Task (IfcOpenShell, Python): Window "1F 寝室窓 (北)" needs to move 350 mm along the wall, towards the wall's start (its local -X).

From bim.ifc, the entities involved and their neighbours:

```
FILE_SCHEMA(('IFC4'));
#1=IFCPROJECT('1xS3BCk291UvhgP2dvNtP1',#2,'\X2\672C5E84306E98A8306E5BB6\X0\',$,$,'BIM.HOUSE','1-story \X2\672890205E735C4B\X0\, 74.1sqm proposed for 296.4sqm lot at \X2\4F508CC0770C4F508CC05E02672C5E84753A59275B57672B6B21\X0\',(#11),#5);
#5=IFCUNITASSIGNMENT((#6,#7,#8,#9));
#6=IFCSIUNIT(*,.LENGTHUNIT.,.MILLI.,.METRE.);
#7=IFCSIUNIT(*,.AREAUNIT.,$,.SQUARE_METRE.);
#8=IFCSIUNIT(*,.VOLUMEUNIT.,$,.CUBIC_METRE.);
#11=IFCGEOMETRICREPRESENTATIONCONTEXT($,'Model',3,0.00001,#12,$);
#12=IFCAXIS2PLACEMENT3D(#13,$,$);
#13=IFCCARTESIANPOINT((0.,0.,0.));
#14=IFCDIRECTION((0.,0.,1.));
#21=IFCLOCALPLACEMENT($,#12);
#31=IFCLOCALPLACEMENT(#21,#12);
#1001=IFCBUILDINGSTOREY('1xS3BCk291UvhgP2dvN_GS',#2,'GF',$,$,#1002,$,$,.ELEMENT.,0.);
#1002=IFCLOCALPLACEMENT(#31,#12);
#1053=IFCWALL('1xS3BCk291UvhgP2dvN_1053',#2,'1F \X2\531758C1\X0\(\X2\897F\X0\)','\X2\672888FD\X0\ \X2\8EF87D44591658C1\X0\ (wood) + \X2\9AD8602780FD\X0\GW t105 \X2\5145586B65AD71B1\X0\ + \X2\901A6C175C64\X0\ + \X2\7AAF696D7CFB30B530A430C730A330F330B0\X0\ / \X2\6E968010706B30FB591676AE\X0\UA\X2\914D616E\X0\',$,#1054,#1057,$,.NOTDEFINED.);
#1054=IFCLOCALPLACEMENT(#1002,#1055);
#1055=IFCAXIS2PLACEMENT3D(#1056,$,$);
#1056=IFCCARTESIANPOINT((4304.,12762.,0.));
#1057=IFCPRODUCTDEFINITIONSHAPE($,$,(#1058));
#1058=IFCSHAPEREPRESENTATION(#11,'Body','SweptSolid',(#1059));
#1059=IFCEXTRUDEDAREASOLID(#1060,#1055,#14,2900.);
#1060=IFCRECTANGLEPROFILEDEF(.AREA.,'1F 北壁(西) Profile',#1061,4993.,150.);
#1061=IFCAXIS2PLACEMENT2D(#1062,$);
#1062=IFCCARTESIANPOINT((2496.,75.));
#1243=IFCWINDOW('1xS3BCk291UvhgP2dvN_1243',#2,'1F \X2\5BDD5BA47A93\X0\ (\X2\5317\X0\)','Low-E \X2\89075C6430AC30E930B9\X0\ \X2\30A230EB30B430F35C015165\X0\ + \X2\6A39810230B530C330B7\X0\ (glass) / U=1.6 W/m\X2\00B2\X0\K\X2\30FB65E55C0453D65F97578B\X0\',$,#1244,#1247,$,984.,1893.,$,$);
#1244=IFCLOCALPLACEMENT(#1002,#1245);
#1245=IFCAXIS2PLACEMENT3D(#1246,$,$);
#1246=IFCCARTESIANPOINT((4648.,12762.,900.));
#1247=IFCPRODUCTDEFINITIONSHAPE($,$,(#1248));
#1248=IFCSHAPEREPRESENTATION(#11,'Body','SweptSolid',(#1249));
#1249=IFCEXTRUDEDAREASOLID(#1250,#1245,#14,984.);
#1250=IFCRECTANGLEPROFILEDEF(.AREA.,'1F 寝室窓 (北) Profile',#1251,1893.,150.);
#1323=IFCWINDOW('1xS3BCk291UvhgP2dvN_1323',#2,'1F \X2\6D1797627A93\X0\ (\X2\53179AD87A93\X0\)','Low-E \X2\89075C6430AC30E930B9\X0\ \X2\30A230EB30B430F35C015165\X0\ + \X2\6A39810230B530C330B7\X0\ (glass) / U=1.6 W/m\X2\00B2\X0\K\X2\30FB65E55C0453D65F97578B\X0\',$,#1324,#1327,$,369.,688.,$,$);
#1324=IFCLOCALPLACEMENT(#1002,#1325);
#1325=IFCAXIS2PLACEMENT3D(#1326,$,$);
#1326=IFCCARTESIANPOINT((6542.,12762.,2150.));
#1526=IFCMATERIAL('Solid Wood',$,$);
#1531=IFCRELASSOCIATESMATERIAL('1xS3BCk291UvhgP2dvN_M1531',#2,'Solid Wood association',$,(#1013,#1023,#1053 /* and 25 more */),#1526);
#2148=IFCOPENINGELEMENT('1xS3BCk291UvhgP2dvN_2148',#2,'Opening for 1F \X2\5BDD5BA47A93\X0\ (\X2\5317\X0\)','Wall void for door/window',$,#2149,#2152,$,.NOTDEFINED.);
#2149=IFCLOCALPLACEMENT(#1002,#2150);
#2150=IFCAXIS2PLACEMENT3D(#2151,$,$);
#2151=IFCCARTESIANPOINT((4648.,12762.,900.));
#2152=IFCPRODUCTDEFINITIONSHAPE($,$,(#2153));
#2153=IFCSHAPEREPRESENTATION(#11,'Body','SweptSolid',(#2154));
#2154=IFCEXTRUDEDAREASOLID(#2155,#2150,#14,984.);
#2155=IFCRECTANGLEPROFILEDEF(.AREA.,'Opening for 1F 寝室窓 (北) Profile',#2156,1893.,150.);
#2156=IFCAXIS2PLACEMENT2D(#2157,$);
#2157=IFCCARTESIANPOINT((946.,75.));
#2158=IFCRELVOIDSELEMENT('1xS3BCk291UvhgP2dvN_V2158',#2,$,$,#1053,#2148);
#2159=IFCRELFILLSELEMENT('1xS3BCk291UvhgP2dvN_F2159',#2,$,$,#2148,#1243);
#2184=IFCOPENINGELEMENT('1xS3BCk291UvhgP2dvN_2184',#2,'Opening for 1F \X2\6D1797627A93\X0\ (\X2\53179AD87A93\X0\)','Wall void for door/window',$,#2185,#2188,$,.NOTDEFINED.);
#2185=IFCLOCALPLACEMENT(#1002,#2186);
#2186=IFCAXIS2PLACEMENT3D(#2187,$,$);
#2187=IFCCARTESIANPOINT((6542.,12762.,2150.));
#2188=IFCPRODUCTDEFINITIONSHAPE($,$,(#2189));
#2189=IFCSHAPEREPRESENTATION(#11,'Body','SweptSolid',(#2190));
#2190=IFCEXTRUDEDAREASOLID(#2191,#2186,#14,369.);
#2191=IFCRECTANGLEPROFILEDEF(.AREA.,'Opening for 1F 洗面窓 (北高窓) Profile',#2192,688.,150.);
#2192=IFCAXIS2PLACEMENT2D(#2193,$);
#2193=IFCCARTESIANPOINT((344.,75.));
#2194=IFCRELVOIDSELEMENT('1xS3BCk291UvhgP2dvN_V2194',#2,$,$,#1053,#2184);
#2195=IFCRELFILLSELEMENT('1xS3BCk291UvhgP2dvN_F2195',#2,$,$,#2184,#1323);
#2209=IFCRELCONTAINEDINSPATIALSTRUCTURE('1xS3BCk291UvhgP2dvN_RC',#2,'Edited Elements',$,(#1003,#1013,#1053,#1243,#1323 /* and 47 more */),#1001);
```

```python
import ifcopenshell
import ifcopenshell.api.geometry
import ifcopenshell.util.placement

model = ifcopenshell.open("bim.ifc")

window = model.by_guid("1xS3BCk291UvhgP2dvN_1243")
opening = window.FillsVoids[0].RelatingOpeningElement
wall = opening.VoidsElements[0].RelatingBuildingElement

wall_matrix = ifcopenshell.util.placement.get_local_placement(wall.ObjectPlacement)
shift = wall_matrix[:3, 0] * -350.0
before = ifcopenshell.util.placement.get_local_placement(window.ObjectPlacement)[:3, 3].copy()

# The window is not placed relative to its opening, so move both.
for product in (opening, window):
    matrix = ifcopenshell.util.placement.get_local_placement(product.ObjectPlacement)
    matrix[:3, 3] += shift
    ifcopenshell.api.geometry.edit_object_placement(model, product=product, matrix=matrix, is_si=False)

after = ifcopenshell.util.placement.get_local_placement(window.ObjectPlacement)[:3, 3]
print("window moved by", (after - before).round(3) + 0.0)

model.write("bim_updated.ifc")
```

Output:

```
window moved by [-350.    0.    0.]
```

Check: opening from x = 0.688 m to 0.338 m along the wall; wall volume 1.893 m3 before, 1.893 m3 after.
